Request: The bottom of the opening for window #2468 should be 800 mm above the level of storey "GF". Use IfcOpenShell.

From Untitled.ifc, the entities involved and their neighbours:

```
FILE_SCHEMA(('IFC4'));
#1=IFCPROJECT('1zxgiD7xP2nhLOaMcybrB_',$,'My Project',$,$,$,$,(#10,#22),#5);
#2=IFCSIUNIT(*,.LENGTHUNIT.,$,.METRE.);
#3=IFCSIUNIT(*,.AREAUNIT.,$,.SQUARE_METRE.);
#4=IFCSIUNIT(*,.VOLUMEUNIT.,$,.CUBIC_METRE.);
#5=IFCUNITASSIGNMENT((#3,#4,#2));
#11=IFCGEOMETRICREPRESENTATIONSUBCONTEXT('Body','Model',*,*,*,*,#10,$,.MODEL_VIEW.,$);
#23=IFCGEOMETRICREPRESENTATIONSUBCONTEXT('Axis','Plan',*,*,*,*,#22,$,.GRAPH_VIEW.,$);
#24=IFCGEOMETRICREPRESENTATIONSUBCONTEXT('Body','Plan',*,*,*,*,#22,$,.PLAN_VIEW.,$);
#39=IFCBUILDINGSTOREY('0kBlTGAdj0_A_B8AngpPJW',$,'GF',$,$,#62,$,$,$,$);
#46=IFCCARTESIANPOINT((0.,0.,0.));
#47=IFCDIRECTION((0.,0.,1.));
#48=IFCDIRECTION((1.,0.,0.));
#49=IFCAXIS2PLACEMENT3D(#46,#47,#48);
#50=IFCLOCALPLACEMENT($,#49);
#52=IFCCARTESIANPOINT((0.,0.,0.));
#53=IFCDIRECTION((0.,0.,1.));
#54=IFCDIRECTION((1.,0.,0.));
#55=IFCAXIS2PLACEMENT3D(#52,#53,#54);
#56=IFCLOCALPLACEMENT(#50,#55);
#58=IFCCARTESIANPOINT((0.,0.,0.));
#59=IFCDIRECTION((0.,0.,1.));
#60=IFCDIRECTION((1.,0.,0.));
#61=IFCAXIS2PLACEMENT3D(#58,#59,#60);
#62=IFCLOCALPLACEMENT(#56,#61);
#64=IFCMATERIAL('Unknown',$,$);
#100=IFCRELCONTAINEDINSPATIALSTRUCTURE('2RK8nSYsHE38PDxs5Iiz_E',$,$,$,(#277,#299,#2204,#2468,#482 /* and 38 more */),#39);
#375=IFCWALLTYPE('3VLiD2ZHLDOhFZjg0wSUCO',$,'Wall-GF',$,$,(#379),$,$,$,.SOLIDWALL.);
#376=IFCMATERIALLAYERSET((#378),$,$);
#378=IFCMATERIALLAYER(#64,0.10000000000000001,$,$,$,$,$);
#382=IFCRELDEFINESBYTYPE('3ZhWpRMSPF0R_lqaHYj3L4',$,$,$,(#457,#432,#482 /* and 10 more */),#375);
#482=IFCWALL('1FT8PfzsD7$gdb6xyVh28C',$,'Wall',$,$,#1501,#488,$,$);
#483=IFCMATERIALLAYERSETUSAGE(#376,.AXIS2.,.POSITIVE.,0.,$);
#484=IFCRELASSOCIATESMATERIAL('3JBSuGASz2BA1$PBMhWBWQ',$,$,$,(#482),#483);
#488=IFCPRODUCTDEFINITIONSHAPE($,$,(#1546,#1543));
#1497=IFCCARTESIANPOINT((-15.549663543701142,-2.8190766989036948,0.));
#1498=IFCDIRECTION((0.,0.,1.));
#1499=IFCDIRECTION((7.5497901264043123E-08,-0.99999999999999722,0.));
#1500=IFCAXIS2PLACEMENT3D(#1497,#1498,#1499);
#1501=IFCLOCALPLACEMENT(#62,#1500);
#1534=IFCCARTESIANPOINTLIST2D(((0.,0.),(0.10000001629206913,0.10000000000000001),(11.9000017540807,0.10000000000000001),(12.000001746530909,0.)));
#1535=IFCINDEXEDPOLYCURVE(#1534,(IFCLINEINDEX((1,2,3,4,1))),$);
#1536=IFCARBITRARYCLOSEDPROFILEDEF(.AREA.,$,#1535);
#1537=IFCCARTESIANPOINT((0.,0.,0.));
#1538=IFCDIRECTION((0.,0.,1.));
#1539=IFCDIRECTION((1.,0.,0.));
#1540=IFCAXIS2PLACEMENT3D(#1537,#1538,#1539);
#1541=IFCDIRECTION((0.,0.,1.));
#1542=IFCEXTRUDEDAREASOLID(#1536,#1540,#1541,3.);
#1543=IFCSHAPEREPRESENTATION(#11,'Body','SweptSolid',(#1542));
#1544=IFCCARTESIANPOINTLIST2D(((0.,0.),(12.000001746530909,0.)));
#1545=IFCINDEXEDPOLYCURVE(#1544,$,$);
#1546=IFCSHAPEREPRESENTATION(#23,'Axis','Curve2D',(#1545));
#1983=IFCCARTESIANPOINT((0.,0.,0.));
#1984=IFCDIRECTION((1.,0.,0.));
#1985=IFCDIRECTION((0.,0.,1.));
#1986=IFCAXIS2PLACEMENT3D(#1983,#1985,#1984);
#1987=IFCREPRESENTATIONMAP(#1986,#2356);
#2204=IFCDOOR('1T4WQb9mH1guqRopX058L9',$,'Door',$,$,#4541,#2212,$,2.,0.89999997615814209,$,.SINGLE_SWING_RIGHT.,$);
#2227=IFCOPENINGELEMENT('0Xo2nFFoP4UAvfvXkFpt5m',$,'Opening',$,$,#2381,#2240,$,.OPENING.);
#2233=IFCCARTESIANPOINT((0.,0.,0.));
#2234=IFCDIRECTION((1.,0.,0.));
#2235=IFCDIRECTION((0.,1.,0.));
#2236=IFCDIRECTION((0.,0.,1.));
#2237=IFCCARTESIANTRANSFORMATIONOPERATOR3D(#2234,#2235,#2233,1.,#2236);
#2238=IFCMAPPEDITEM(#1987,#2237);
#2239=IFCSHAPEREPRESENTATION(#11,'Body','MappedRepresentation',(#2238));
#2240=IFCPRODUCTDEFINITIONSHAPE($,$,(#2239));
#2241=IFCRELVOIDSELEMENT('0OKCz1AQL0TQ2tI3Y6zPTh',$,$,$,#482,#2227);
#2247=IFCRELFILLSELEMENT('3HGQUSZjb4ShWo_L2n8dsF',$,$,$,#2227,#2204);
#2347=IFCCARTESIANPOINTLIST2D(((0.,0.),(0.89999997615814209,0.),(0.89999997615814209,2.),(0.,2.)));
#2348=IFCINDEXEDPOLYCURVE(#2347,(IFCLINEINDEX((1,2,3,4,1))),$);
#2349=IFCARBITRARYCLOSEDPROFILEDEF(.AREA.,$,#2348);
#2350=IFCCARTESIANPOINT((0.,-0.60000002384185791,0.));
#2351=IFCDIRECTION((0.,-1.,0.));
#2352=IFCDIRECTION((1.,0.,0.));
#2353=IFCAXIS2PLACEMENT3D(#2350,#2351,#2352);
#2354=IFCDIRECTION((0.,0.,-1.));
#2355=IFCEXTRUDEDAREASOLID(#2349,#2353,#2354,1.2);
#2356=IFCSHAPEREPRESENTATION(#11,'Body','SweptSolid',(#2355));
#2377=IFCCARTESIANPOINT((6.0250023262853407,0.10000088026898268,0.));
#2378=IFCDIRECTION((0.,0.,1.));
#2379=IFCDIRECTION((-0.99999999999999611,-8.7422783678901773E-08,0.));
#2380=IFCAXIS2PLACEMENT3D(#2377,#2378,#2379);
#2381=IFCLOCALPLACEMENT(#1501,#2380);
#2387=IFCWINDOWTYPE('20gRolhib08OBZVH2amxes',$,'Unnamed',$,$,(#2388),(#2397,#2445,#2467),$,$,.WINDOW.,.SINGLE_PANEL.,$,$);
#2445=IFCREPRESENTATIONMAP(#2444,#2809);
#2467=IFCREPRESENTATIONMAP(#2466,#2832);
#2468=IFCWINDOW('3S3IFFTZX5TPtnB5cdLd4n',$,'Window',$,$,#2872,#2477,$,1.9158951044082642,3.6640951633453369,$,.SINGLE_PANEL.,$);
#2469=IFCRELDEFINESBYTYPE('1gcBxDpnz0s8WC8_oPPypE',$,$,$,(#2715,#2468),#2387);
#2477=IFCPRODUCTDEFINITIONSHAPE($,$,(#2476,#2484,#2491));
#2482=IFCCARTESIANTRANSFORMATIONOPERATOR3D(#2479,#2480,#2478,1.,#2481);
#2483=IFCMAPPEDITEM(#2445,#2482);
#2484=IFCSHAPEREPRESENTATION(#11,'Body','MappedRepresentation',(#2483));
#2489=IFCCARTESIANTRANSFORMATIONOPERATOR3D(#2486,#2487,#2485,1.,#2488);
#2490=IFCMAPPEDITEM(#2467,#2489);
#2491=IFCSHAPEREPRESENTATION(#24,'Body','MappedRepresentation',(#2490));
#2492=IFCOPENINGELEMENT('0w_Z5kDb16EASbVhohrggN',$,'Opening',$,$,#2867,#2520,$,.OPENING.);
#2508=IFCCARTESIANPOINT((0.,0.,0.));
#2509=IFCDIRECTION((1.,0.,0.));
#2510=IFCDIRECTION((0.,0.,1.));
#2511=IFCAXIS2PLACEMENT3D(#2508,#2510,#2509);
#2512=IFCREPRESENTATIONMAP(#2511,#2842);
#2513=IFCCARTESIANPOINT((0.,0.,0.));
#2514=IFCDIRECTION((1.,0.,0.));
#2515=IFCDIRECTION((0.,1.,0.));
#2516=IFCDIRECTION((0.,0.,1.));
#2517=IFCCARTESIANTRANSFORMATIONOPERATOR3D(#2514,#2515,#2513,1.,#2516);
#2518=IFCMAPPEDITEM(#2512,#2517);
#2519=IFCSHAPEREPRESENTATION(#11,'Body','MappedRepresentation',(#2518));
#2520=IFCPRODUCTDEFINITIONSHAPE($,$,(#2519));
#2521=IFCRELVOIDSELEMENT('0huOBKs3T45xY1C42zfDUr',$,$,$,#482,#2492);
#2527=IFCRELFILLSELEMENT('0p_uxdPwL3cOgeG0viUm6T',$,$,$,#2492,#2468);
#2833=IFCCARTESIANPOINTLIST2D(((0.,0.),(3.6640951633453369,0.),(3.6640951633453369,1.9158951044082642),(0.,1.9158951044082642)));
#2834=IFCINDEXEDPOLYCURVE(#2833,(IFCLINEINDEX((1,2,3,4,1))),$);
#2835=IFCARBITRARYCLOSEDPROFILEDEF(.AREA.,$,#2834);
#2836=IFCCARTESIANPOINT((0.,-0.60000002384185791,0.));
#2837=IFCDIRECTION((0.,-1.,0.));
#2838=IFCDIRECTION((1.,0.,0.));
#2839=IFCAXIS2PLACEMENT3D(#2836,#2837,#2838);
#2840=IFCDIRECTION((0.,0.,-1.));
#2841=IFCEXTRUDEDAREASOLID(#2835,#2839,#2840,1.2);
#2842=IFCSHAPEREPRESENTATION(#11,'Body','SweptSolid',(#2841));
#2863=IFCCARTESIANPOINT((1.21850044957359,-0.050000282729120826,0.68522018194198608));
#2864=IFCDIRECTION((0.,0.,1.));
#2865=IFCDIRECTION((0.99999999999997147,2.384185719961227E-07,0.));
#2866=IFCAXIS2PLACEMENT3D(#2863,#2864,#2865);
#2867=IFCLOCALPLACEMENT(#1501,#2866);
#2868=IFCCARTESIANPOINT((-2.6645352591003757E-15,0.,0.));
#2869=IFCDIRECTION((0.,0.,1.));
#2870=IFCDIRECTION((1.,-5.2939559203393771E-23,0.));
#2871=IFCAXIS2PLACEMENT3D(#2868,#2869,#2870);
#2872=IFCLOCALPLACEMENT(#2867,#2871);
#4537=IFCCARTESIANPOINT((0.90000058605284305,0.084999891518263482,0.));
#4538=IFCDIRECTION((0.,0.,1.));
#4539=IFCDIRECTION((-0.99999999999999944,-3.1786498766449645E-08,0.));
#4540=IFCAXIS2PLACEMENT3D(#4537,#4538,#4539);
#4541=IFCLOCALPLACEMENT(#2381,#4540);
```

```python
import numpy as np
import ifcopenshell
import ifcopenshell.api.geometry
import ifcopenshell.geom
import ifcopenshell.util.element
import ifcopenshell.util.placement
import ifcopenshell.util.shape
import ifcopenshell.util.unit

model = ifcopenshell.open("Untitled.ifc")
unit_scale = ifcopenshell.util.unit.calculate_unit_scale(model)

window = model.by_guid("3S3IFFTZX5TPtnB5cdLd4n")
opening = window.FillsVoids[0].RelatingOpeningElement
storey = ifcopenshell.util.element.get_container(window, ifc_class="IfcBuildingStorey")
level = ifcopenshell.util.placement.get_local_placement(storey.ObjectPlacement)[2, 3]

# The opening's origin need not be at the sill, so measure its lowest point.
shape = ifcopenshell.geom.create_shape(ifcopenshell.geom.settings(), opening)
bottom = ifcopenshell.util.shape.get_shape_bottom_elevation(shape, shape.geometry) / unit_scale
dz = level + 0.8 - bottom

shift = np.array([0.0, 0.0, dz])
# The window is placed relative to its opening, so it follows when the opening moves.
matrix = ifcopenshell.util.placement.get_local_placement(opening.ObjectPlacement)
matrix[:3, 3] += shift
ifcopenshell.api.geometry.edit_object_placement(
    model, product=opening, matrix=matrix, is_si=False, should_transform_children=True
)

print(f"moved by {dz * unit_scale:+.3f} m")

model.write("Untitled-out.ifc")
```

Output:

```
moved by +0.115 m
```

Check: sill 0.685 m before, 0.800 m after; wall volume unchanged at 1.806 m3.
